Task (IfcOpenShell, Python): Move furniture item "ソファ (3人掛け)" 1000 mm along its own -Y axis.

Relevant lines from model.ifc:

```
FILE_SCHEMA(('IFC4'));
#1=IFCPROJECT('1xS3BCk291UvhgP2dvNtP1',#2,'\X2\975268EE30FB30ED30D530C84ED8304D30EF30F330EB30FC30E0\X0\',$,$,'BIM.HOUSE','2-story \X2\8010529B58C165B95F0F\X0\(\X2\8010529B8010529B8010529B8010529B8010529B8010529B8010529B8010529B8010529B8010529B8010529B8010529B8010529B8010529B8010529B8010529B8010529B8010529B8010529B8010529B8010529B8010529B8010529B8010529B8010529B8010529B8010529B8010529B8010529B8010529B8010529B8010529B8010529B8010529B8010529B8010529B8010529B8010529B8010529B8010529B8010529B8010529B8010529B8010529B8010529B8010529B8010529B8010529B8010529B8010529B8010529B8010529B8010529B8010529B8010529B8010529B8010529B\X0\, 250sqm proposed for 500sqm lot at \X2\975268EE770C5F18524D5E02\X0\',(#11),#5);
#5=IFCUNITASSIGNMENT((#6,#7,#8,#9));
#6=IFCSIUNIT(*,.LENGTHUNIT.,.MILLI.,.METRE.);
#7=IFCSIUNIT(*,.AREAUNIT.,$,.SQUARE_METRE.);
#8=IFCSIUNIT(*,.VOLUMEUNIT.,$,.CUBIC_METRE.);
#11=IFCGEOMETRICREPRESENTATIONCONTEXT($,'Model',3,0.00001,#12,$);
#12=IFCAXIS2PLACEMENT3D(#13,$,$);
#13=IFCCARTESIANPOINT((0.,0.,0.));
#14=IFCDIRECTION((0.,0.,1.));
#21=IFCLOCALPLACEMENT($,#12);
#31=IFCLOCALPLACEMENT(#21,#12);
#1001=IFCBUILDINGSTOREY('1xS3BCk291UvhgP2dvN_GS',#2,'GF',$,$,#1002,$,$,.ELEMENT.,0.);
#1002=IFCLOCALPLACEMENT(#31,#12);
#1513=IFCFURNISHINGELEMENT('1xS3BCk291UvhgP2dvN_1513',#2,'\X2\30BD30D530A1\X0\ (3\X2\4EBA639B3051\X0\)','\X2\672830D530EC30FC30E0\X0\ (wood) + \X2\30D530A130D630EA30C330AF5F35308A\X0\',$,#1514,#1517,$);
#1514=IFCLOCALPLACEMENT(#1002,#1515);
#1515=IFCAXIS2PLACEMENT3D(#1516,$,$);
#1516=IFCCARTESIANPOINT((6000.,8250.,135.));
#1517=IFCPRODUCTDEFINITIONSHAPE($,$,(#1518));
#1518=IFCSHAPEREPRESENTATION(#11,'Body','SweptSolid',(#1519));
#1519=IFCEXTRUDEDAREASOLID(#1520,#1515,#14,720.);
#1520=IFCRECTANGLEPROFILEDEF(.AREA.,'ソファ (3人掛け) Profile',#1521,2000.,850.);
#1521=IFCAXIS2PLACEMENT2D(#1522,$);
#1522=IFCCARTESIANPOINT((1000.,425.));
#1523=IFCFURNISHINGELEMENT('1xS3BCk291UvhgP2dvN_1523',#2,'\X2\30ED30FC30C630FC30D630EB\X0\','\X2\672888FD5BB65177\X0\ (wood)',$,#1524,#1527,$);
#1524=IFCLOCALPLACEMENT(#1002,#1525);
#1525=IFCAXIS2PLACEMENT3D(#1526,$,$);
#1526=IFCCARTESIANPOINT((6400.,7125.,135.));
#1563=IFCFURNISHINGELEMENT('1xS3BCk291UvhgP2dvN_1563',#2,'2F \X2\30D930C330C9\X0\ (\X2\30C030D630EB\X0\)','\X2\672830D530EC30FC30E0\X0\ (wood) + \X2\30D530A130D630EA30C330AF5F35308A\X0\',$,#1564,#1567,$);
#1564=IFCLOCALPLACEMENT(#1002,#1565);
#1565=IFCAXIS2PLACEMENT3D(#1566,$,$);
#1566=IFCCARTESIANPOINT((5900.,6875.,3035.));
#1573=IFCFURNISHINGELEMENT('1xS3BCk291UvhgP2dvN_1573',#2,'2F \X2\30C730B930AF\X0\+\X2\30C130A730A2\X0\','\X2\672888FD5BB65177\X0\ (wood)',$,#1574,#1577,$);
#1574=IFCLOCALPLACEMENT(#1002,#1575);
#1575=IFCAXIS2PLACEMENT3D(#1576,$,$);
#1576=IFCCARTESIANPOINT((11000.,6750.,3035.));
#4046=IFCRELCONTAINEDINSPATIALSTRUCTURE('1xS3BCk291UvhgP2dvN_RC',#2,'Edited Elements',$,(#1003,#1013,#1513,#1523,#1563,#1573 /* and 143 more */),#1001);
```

```python
import ifcopenshell
import ifcopenshell.api.geometry
import ifcopenshell.util.placement

model = ifcopenshell.open("model.ifc")

item = model.by_guid("1xS3BCk291UvhgP2dvN_1513")
matrix = ifcopenshell.util.placement.get_local_placement(item.ObjectPlacement)
matrix[:3, 3] -= matrix[:3, 1] * 1000.0
ifcopenshell.api.geometry.edit_object_placement(model, product=item, matrix=matrix, is_si=False)

print(ifcopenshell.util.placement.get_local_placement(item.ObjectPlacement).round(3) + 0.0)

model.write("model-out.ifc")
```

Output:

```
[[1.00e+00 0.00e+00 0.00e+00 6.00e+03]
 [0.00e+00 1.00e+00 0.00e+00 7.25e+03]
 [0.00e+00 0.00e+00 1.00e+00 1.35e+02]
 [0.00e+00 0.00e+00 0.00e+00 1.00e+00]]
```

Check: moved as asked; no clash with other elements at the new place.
